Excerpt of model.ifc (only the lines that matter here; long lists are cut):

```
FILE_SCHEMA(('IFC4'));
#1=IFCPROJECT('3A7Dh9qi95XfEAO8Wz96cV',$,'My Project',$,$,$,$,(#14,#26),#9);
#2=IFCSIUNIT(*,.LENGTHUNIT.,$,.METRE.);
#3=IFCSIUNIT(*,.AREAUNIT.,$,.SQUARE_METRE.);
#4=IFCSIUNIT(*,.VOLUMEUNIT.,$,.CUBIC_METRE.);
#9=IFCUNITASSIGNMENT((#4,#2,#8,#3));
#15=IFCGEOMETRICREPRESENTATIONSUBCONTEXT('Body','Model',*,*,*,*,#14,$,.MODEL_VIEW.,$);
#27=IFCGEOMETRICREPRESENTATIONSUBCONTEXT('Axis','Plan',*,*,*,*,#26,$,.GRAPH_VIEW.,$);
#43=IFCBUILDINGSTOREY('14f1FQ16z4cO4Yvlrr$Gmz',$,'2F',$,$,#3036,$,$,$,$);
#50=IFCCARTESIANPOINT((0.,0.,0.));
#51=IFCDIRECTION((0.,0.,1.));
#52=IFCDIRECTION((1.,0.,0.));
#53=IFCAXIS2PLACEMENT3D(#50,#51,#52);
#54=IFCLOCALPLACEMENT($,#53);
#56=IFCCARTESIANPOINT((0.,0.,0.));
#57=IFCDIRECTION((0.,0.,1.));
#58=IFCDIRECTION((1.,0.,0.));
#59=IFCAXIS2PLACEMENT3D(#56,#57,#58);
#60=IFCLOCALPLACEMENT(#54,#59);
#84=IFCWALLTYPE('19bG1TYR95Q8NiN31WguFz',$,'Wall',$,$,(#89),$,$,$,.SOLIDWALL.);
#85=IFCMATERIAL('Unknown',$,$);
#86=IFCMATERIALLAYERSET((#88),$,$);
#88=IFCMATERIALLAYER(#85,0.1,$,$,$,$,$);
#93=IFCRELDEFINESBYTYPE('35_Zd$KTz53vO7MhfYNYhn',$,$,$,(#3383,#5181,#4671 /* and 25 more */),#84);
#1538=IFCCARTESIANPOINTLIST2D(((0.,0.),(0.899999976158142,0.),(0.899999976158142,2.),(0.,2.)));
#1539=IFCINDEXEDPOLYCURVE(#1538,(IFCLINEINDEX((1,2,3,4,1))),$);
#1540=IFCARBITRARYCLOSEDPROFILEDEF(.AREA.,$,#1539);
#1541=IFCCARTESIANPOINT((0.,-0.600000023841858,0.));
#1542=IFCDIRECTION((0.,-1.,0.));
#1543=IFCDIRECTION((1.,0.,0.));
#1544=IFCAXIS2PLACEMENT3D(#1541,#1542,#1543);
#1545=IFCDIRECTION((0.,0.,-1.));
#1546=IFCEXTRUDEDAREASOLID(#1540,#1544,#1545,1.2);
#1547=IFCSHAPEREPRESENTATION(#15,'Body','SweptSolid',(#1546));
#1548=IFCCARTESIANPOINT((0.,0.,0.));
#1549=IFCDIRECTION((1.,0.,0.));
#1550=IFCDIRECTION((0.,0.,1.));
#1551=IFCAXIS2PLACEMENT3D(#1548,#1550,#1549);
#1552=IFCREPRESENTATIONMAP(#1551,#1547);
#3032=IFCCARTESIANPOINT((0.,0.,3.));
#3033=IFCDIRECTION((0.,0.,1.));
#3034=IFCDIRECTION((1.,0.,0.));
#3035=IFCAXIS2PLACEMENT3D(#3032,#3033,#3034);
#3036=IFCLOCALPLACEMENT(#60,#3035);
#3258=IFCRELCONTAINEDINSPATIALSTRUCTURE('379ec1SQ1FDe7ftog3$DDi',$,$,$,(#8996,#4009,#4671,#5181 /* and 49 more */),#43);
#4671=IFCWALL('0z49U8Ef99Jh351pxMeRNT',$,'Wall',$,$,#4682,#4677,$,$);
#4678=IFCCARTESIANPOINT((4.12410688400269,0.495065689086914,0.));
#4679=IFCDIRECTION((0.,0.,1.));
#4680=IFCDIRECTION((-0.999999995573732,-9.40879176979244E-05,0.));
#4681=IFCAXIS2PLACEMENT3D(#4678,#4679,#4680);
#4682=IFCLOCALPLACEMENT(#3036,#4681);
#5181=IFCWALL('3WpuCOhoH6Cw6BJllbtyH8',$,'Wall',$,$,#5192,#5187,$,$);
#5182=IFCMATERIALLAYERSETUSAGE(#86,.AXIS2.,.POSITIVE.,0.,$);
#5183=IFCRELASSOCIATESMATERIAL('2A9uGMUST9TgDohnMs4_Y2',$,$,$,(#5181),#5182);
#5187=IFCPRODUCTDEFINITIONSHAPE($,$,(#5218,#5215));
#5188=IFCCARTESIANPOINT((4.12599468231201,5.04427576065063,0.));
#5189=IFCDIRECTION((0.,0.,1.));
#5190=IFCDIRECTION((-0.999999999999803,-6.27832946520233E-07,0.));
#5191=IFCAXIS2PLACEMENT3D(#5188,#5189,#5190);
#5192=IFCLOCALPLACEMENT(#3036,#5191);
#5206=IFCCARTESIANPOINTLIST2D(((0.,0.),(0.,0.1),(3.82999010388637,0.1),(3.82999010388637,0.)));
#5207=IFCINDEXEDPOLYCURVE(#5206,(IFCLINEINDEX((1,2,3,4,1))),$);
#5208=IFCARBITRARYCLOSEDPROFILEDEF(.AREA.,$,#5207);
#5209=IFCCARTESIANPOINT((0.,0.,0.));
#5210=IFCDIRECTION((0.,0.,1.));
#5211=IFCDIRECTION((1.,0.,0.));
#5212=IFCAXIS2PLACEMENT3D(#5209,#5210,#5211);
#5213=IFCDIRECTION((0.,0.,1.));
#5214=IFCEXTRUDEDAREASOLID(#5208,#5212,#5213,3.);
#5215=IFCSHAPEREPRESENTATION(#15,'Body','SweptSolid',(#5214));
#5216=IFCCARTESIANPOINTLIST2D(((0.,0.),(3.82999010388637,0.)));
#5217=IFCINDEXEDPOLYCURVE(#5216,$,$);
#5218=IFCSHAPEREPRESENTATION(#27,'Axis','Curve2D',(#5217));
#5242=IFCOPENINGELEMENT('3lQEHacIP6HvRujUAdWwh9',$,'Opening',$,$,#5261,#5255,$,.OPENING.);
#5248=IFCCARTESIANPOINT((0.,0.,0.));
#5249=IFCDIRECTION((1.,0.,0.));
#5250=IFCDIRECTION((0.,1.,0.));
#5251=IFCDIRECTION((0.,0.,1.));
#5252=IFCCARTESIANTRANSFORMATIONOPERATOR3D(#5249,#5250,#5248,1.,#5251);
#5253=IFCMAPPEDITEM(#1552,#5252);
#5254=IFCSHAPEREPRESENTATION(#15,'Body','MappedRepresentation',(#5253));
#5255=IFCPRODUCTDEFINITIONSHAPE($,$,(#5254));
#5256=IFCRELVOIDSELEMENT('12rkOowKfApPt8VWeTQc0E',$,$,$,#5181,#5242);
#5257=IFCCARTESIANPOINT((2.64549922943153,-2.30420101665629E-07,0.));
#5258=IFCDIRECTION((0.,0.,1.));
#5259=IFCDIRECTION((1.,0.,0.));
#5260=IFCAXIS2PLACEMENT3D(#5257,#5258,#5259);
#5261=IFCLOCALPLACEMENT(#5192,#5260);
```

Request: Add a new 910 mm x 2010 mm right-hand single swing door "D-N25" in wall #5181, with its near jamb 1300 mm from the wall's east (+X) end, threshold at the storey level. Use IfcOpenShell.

```python
import numpy as np
import ifcopenshell
import ifcopenshell.api.feature
import ifcopenshell.api.geometry
import ifcopenshell.api.root
import ifcopenshell.api.spatial
import ifcopenshell.geom
import ifcopenshell.util.element
import ifcopenshell.util.placement
import ifcopenshell.util.representation
import ifcopenshell.util.shape
import ifcopenshell.util.unit

model = ifcopenshell.open("model.ifc")
unit_scale = ifcopenshell.util.unit.calculate_unit_scale(model)
settings = ifcopenshell.geom.settings()


def volume(element):
    """Net volume in cubic metres, openings subtracted."""
    shape = ifcopenshell.geom.create_shape(settings, element)
    return ifcopenshell.util.shape.get_volume(shape.geometry)


wall = model.by_guid("3WpuCOhoH6Cw6BJllbtyH8")
storey = ifcopenshell.util.element.get_container(wall, ifc_class="IfcBuildingStorey")
context = ifcopenshell.util.representation.get_context(model, "Model", "Body", "MODEL_VIEW")
before = volume(wall)

width, height, from_end, sill = 0.91, 2.01, 1.3, 0.0  # metres

# The wall runs along its own X axis, and the end named is its -X end.
wall_shape = ifcopenshell.geom.create_shape(settings, wall)
x, y, z = ifcopenshell.util.shape.get_vertices(wall_shape.geometry).T
start = x.min() + from_end
face, thickness = float(y.min()), float(y.max() - y.min())
wall_matrix = ifcopenshell.util.placement.get_local_placement(wall.ObjectPlacement)
level = ifcopenshell.util.placement.get_local_placement(storey.ObjectPlacement)[2, 3]


def in_wall(x, y):
    """Placement at x, y metres in the wall's axes, at sill height."""
    matrix = wall_matrix.copy()
    matrix[:, 3] = wall_matrix @ np.array([x / unit_scale, y / unit_scale, 0.0, 1.0])
    matrix[2, 3] = level + sill / unit_scale
    return matrix


# Opening: a box that overshoots both wall faces by 50 mm.
opening = ifcopenshell.api.root.create_entity(model, ifc_class="IfcOpeningElement", predefined_type="OPENING")
box = ifcopenshell.api.geometry.add_wall_representation(
    model, context=context, length=width, height=height, thickness=thickness + 0.1
)
ifcopenshell.api.geometry.assign_representation(model, product=opening, representation=box)
ifcopenshell.api.geometry.edit_object_placement(model, product=opening, matrix=in_wall(start, face - 0.05), is_si=False)
ifcopenshell.api.feature.add_feature(model, feature=opening, element=wall)

door = ifcopenshell.api.root.create_entity(model, ifc_class="IfcDoor", name="D-N25", predefined_type="DOOR")
door.OverallWidth, door.OverallHeight = width / unit_scale, height / unit_scale
door.OperationType = "SINGLE_SWING_RIGHT"
body = ifcopenshell.api.geometry.add_door_representation(
    model,
    context=context,
    overall_width=door.OverallWidth,
    overall_height=door.OverallHeight,
    operation_type="SINGLE_SWING_RIGHT",
    lining_properties={"LiningDepth": thickness / unit_scale, "ThresholdDepth": thickness / unit_scale},
)
ifcopenshell.api.geometry.assign_representation(model, product=door, representation=body)
ifcopenshell.api.spatial.assign_container(model, products=[door], relating_structure=storey)
ifcopenshell.api.feature.add_filling(model, opening=opening, element=door)

# The lining spans the wall, so the door starts at the wall face.
ifcopenshell.api.geometry.edit_object_placement(model, product=door, matrix=in_wall(start, face), is_si=False)

after = volume(wall)

print(f"wall volume {before:.3f} -> {after:.3f} m3")

model.write("model_v2.ifc")
```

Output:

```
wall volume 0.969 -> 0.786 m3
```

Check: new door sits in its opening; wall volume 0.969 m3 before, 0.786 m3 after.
